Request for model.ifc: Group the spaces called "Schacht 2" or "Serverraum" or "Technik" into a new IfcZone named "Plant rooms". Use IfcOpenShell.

First a look at what the model holds.

```python
import ifcopenshell

model = ifcopenshell.open("model.ifc")
print(model.schema)
seen = {}
for space in model.by_type("IfcSpace"):
    seen[space.LongName] = seen.get(space.LongName, 0) + 1
for name, count in sorted(seen.items(), key=str):
    print(count, "x", name)
print("zones:", [z.Name for z in model.by_type("IfcZone")][:20])
```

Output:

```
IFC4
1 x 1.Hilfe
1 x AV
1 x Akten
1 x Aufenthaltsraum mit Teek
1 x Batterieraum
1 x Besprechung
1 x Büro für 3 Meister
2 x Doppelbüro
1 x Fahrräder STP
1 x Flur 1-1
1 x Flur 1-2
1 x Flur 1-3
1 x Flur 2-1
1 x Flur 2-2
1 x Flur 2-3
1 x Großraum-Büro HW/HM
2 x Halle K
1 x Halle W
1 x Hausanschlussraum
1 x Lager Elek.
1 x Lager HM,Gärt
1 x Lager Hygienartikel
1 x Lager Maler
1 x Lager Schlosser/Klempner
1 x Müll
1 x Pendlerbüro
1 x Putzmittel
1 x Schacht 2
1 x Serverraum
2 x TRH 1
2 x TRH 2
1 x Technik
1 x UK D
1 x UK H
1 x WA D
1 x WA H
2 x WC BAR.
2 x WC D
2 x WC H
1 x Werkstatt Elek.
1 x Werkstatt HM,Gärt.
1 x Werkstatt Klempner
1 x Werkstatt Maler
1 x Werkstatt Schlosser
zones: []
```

```python
import ifcopenshell
import ifcopenshell.api.group
import ifcopenshell.api.root

model = ifcopenshell.open("model.ifc")

names = {"Schacht 2", "Serverraum", "Technik"}
spaces = [s for s in model.by_type("IfcSpace") if s.LongName in names]

zone = ifcopenshell.api.root.create_entity(model, ifc_class="IfcZone", name="Plant rooms")
ifcopenshell.api.group.assign_group(model, products=spaces, group=zone)
print(len(spaces), "spaces in", zone.Name)

model.write("model-out.ifc")
```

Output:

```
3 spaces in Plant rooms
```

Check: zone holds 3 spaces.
